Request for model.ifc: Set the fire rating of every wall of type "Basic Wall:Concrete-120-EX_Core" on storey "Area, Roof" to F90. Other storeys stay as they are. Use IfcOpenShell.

First a look at what the model holds.

```python
import ifcopenshell
import ifcopenshell.util.element

model = ifcopenshell.open("model.ifc")
print(model.schema)
storey = next(s for s in model.by_type("IfcBuildingStorey") if s.Name == "Area, Roof")
walls = [e for e in ifcopenshell.util.element.get_decomposition(storey) if e.is_a("IfcWall")]
seen = {}
for e in walls:
    element_type = ifcopenshell.util.element.get_type(e)
    key = (element_type.Name if element_type != e and element_type else None, ifcopenshell.util.element.get_pset(e, "Pset_WallCommon", "FireRating"))
    seen[key] = seen.get(key, 0) + 1
for (name, value), count in sorted(seen.items(), key=str):
    print(count, "x", name, "|", value)
```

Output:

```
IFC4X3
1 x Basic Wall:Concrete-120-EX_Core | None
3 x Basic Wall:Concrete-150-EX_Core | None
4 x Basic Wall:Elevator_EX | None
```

```python
import ifcopenshell
import ifcopenshell.api.pset
import ifcopenshell.util.element

model = ifcopenshell.open("model.ifc")

storey = next(s for s in model.by_type("IfcBuildingStorey") if s.Name == "Area, Roof")
walls = [e for e in ifcopenshell.util.element.get_decomposition(storey) if e.is_a("IfcWall")]

count = 0
for e in walls:
    element_type = ifcopenshell.util.element.get_type(e)
    if element_type in (None, e) or element_type.Name != "Basic Wall:Concrete-120-EX_Core":
        continue
    # add_pset returns the element's existing set when there is one.
    pset = ifcopenshell.api.pset.add_pset(model, product=e, name="Pset_WallCommon")
    ifcopenshell.api.pset.edit_pset(model, pset=pset, properties={"FireRating": "F90"})
    count += 1

print(count, "walls updated")

model.write("model-out.ifc")
```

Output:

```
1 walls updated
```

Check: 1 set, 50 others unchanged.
